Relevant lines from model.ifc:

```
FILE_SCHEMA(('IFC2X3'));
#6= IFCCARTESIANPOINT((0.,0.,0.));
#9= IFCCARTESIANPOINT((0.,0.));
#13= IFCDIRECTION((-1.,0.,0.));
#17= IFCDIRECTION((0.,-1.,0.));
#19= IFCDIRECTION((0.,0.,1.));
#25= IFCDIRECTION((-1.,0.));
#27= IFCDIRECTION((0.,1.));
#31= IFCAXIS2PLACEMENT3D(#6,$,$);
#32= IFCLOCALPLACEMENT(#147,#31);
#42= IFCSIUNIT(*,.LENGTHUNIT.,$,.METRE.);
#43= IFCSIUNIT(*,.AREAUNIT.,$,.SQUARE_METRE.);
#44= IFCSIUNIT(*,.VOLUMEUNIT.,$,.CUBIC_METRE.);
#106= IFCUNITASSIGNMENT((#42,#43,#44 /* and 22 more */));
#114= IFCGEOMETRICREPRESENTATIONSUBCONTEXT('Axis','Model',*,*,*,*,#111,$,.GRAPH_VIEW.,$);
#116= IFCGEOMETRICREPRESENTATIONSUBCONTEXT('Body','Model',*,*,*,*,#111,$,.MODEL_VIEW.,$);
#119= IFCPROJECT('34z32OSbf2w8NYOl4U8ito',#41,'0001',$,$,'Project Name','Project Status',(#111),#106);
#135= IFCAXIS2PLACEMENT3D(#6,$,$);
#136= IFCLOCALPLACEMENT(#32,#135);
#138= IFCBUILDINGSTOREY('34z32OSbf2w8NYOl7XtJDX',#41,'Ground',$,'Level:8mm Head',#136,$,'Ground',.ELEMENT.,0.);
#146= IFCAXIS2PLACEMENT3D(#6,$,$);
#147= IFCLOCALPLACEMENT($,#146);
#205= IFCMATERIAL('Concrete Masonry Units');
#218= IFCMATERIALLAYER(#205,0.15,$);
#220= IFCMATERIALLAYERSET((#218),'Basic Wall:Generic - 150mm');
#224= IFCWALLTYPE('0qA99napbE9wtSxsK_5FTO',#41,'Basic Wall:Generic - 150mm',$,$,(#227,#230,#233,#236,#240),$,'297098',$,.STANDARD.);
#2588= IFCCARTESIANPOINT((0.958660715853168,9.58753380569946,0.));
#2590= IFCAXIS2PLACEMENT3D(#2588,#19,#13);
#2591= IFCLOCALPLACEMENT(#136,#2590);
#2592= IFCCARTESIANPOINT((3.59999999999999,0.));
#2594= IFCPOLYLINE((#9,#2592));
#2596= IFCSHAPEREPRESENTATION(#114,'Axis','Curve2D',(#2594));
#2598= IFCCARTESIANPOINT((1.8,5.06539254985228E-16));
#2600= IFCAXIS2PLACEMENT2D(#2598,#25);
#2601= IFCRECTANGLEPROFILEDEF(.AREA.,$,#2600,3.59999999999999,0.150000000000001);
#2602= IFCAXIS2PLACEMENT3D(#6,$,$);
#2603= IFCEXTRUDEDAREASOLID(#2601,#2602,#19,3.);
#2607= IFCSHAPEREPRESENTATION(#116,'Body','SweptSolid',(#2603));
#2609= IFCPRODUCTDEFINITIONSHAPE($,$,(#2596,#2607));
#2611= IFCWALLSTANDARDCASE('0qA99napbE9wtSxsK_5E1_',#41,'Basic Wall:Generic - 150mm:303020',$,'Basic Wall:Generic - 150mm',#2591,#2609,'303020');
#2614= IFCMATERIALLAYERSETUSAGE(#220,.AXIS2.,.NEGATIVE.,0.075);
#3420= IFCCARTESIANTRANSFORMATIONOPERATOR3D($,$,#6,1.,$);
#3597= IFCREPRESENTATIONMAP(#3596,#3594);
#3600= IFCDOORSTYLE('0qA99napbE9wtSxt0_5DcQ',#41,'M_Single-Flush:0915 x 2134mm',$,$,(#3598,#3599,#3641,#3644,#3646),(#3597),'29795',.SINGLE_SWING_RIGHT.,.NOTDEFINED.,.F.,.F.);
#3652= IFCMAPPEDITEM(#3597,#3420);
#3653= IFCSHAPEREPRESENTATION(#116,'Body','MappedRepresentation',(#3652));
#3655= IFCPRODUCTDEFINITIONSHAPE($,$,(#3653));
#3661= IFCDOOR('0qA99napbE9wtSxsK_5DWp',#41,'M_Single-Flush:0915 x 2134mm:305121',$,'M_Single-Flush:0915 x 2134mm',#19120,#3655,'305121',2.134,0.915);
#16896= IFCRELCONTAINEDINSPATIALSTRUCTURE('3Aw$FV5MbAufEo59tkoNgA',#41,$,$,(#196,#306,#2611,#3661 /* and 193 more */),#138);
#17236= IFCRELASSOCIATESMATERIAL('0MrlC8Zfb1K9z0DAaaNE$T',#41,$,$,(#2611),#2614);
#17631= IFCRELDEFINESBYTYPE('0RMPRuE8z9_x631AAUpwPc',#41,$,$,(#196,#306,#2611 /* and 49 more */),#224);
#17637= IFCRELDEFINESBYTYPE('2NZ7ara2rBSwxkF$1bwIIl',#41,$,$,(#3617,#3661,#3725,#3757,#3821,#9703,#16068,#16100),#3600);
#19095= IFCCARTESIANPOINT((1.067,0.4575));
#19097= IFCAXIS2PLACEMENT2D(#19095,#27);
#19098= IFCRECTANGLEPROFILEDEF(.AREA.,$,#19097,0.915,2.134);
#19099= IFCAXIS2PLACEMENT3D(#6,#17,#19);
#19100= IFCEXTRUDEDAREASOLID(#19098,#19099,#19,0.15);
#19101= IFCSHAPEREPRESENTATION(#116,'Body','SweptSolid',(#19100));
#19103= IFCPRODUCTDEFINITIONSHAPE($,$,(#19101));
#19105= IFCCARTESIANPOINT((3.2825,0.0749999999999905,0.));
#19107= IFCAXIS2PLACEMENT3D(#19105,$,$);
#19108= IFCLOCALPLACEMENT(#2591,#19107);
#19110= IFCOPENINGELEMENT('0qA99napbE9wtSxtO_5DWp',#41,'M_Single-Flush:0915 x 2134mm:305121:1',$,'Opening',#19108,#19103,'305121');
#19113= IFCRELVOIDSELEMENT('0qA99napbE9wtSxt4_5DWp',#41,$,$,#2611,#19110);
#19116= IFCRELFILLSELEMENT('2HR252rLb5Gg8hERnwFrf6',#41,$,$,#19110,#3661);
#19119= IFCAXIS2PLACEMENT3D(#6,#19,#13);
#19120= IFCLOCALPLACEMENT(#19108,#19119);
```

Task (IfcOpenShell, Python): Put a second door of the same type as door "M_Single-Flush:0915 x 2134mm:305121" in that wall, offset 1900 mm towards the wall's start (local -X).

```python
import ifcopenshell
import ifcopenshell.api.feature
import ifcopenshell.api.geometry
import ifcopenshell.api.root
import ifcopenshell.geom
import ifcopenshell.util.element
import ifcopenshell.util.placement
import ifcopenshell.util.shape
import ifcopenshell.util.unit

model = ifcopenshell.open("model.ifc")
unit_scale = ifcopenshell.util.unit.calculate_unit_scale(model)
settings = ifcopenshell.geom.settings()


def volume(element):
    """Net volume in cubic metres, openings subtracted."""
    shape = ifcopenshell.geom.create_shape(settings, element)
    return ifcopenshell.util.shape.get_volume(shape.geometry)


def reuse_history(source, copy):
    """copy_class also copies each property set's owner history, people and application; keep the originals."""
    for rel in copy.IsDefinedBy:
        if rel.is_a("IfcRelDefinesByProperties") and (history := rel.RelatingPropertyDefinition.OwnerHistory):
            rel.RelatingPropertyDefinition.OwnerHistory = source.OwnerHistory
            ifcopenshell.util.element.remove_deep2(model, history)


door = model.by_guid("0qA99napbE9wtSxsK_5DWp")
opening = door.FillsVoids[0].RelatingOpeningElement
wall = opening.VoidsElements[0].RelatingBuildingElement
before = volume(wall)
shift = ifcopenshell.util.placement.get_local_placement(wall.ObjectPlacement)[:3, 0] * -1.9 / unit_scale

# copy_class copies the void relationship, type, container and properties, but no geometry.
new_opening = ifcopenshell.api.root.copy_class(model, product=opening)
new_opening.Representation = ifcopenshell.util.element.copy_deep(
    model, opening.Representation, exclude=["IfcGeometricRepresentationContext", "IfcRepresentationMap"]
)
new_opening.Name = "M_Single-Flush:0915 x 2134mm"
new_opening.Tag = None
new_door = ifcopenshell.api.root.copy_class(model, product=door)
new_door.Representation = ifcopenshell.util.element.copy_deep(
    model, door.Representation, exclude=["IfcGeometricRepresentationContext", "IfcRepresentationMap"]
)
new_door.Name = "M_Single-Flush:0915 x 2134mm"
new_door.Tag = None
reuse_history(door, new_door)
fills = ifcopenshell.api.feature.add_filling(model, opening=new_opening, element=new_door)
fills.OwnerHistory = new_door.OwnerHistory  # required in IFC2X3

for old, new in ((opening, new_opening), (door, new_door)):
    matrix = ifcopenshell.util.placement.get_local_placement(old.ObjectPlacement)
    matrix[:3, 3] += shift
    ifcopenshell.api.geometry.edit_object_placement(model, product=new, matrix=matrix, is_si=False)

after = volume(wall)

print(f"wall volume {before:.3f} -> {after:.3f} m3")

model.write("model_v2.ifc")
```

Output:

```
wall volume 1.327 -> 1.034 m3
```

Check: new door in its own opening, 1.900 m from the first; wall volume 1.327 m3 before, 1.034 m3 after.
